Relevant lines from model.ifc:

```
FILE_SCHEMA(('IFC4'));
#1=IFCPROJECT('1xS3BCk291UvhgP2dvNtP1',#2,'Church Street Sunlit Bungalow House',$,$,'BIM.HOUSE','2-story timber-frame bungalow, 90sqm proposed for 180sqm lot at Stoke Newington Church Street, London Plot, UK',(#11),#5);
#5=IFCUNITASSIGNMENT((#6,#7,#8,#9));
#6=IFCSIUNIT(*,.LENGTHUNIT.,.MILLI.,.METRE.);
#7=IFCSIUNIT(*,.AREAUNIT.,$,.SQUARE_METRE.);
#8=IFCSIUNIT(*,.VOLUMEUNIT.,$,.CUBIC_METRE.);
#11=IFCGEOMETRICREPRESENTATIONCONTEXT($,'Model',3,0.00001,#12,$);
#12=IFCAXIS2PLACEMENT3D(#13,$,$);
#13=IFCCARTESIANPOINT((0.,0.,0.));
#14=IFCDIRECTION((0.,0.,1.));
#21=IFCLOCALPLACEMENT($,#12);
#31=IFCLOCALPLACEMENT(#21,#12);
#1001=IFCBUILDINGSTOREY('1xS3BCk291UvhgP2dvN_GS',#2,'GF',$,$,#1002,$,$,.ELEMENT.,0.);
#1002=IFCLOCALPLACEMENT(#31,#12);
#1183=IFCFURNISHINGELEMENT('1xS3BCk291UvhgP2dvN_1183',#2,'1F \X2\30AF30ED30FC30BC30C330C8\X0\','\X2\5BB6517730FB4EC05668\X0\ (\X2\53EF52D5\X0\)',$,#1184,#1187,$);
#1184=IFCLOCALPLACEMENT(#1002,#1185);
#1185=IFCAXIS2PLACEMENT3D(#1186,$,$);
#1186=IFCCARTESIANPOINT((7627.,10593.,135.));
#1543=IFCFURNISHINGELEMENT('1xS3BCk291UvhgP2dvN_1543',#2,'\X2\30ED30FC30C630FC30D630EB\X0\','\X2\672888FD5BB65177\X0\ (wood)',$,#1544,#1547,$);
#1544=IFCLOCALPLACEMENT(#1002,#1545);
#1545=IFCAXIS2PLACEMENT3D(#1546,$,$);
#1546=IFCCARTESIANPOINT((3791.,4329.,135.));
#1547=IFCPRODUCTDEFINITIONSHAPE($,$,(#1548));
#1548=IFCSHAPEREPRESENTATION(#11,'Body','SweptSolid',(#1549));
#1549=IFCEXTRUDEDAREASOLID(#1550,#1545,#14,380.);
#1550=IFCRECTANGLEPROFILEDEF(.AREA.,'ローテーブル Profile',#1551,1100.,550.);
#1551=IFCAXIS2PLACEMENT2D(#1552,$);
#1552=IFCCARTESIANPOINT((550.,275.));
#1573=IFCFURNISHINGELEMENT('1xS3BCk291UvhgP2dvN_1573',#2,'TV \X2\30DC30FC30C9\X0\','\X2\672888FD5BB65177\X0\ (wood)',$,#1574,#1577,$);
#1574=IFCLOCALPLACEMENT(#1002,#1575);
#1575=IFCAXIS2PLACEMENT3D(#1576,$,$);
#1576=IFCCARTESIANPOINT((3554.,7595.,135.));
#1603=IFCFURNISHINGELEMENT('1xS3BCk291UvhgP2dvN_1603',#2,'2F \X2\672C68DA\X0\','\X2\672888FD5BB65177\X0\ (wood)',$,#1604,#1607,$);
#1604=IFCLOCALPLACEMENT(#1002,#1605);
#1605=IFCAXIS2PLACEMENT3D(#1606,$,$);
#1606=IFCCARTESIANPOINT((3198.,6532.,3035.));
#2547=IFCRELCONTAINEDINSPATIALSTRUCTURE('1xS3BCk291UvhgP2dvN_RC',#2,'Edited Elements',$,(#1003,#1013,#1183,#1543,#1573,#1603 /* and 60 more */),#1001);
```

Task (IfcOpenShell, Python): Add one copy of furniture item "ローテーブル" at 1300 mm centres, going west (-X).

```python
import numpy as np
import ifcopenshell
import ifcopenshell.api.geometry
import ifcopenshell.api.root
import ifcopenshell.util.element
import ifcopenshell.util.placement
import ifcopenshell.util.unit

model = ifcopenshell.open("model.ifc")
unit_scale = ifcopenshell.util.unit.calculate_unit_scale(model)


def reuse_history(source, copy):
    """copy_class also copies each property set's owner history, people and application; keep the originals."""
    for rel in copy.IsDefinedBy:
        if rel.is_a("IfcRelDefinesByProperties") and (history := rel.RelatingPropertyDefinition.OwnerHistory):
            rel.RelatingPropertyDefinition.OwnerHistory = source.OwnerHistory
            ifcopenshell.util.element.remove_deep2(model, history)


source = model.by_guid("1xS3BCk291UvhgP2dvN_1543")
base = ifcopenshell.util.placement.get_local_placement(source.ObjectPlacement)
step = np.array([-1.0, 0.0, 0.0]) * 1.3 / unit_scale

for i in range(1, 2):
    copy = ifcopenshell.api.root.copy_class(model, product=source)
    copy.Representation = ifcopenshell.util.element.copy_deep(
        model, source.Representation, exclude=["IfcGeometricRepresentationContext", "IfcRepresentationMap"]
    )
    reuse_history(source, copy)
    matrix = base.copy()
    matrix[:3, 3] += i * step
    print("added at", matrix[:3, 3].round(3) + 0.0)
    ifcopenshell.api.geometry.edit_object_placement(model, product=copy, matrix=matrix, is_si=False)

model.write("model_v2.ifc")
```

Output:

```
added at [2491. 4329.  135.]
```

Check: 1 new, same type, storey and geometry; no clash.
